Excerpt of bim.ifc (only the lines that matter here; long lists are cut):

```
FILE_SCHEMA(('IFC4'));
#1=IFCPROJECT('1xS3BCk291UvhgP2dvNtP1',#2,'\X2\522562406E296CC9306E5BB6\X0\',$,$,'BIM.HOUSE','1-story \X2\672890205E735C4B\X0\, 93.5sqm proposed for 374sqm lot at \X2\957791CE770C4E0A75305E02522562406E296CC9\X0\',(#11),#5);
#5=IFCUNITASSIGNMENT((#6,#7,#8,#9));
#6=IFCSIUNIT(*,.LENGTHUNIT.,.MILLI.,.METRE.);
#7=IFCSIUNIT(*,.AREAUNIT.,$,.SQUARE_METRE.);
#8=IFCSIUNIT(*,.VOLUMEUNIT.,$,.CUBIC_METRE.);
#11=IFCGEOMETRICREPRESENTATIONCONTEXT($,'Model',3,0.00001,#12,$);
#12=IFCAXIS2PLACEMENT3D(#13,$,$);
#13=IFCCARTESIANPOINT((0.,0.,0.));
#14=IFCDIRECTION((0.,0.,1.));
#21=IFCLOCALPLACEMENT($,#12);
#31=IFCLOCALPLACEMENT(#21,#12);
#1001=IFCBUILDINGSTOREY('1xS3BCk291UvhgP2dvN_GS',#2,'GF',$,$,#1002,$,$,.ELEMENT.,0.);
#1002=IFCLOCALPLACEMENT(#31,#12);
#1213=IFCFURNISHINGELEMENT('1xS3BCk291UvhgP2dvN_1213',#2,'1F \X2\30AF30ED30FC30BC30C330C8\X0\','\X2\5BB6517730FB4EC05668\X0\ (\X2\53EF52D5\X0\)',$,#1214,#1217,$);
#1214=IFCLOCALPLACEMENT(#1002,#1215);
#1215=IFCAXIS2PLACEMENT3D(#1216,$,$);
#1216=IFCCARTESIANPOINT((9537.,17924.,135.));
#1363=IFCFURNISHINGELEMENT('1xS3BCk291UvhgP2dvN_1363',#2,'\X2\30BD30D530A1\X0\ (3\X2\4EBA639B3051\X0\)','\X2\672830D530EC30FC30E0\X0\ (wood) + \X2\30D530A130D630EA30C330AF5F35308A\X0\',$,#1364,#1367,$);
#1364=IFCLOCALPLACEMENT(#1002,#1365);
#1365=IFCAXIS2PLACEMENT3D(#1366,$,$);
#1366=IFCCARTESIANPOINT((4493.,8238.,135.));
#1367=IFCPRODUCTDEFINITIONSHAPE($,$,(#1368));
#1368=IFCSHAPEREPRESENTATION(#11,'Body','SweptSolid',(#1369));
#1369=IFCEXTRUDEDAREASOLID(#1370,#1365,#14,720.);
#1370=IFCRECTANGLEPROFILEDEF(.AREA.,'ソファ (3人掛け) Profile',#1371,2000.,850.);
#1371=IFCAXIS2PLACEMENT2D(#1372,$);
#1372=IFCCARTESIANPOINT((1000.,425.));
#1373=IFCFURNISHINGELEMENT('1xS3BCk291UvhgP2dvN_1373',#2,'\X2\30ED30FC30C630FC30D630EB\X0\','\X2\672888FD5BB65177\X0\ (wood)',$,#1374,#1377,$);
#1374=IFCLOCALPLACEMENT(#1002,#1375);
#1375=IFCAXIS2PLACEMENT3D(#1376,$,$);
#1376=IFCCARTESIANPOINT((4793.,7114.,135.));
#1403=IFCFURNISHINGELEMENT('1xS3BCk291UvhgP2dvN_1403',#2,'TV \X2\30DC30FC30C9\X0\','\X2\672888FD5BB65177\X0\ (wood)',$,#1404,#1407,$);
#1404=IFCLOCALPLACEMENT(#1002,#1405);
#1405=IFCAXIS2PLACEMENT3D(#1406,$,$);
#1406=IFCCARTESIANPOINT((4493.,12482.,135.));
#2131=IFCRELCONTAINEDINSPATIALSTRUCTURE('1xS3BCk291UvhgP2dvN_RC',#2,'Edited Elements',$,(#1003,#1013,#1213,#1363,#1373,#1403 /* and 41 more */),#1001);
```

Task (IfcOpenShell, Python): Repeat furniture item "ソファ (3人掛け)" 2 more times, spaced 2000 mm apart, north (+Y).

```python
import numpy as np
import ifcopenshell
import ifcopenshell.api.geometry
import ifcopenshell.api.root
import ifcopenshell.util.element
import ifcopenshell.util.placement
import ifcopenshell.util.unit

model = ifcopenshell.open("bim.ifc")
unit_scale = ifcopenshell.util.unit.calculate_unit_scale(model)


def reuse_history(source, copy):
    """copy_class also copies each property set's owner history, people and application; keep the originals."""
    for rel in copy.IsDefinedBy:
        if rel.is_a("IfcRelDefinesByProperties") and (history := rel.RelatingPropertyDefinition.OwnerHistory):
            rel.RelatingPropertyDefinition.OwnerHistory = source.OwnerHistory
            ifcopenshell.util.element.remove_deep2(model, history)


source = model.by_id(1363)
base = ifcopenshell.util.placement.get_local_placement(source.ObjectPlacement)
step = np.array([0.0, 1.0, 0.0]) * 2 / unit_scale

for i in range(1, 3):
    copy = ifcopenshell.api.root.copy_class(model, product=source)
    copy.Representation = ifcopenshell.util.element.copy_deep(
        model, source.Representation, exclude=["IfcGeometricRepresentationContext", "IfcRepresentationMap"]
    )
    reuse_history(source, copy)
    matrix = base.copy()
    matrix[:3, 3] += i * step
    print("added at", matrix[:3, 3].round(3) + 0.0)
    ifcopenshell.api.geometry.edit_object_placement(model, product=copy, matrix=matrix, is_si=False)

model.write("bim_rev.ifc")
```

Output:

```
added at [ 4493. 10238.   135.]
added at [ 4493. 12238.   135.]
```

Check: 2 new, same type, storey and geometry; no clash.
